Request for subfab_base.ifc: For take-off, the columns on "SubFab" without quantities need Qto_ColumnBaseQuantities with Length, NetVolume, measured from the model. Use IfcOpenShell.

First a look at what the model holds.

```python
import ifcopenshell
import ifcopenshell.util.element
import ifcopenshell.util.unit

model = ifcopenshell.open("subfab_base.ifc")
print(model.schema)
for unit_type in ("LENGTHUNIT", "AREAUNIT", "VOLUMEUNIT"):
    print(unit_type, ifcopenshell.util.unit.calculate_unit_scale(model, unit_type))
storey = next(s for s in model.by_type("IfcBuildingStorey") if s.Name == "SubFab")
columns = [e for e in ifcopenshell.util.element.get_decomposition(storey) if e.is_a("IfcColumn")]
for e in sorted(columns, key=lambda e: e.id()):
    print(e.id(), e.is_a(), e.Name, list(ifcopenshell.util.element.get_psets(e, qtos_only=True)), sep=" | ")
```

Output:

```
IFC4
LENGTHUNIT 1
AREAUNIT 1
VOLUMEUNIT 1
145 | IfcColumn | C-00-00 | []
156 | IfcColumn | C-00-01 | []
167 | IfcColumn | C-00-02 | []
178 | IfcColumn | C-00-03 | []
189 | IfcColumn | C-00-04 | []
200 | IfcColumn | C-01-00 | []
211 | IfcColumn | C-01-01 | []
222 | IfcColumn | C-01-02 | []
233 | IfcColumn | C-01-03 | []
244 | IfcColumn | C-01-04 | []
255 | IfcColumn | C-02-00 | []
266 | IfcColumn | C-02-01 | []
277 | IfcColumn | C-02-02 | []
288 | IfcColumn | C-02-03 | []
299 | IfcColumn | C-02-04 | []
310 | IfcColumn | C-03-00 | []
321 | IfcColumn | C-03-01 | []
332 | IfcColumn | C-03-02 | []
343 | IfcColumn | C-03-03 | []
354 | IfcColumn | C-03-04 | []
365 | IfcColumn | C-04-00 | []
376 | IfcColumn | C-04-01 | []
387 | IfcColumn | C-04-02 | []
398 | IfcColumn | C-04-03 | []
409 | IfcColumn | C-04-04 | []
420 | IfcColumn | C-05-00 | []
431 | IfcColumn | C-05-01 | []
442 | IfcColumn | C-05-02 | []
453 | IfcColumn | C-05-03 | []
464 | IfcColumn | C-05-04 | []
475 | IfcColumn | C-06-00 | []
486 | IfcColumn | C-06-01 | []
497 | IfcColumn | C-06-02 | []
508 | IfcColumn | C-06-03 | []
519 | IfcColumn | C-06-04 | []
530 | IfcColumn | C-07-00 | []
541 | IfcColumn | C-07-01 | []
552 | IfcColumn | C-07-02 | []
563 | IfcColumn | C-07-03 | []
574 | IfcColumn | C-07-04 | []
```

```python
import ifcopenshell
import ifcopenshell.api.pset
import ifcopenshell.geom
import ifcopenshell.util.element
import ifcopenshell.util.shape
import ifcopenshell.util.unit

model = ifcopenshell.open("subfab_base.ifc")
unit_scale = ifcopenshell.util.unit.calculate_unit_scale(model)
volume_scale = ifcopenshell.util.unit.calculate_unit_scale(model, "VOLUMEUNIT")
settings = ifcopenshell.geom.settings()

storey = next(s for s in model.by_type("IfcBuildingStorey") if s.Name == "SubFab")
columns = [e for e in ifcopenshell.util.element.get_decomposition(storey) if e.is_a("IfcColumn")]

for e in sorted(columns, key=lambda e: e.id()):
    if ifcopenshell.util.element.get_psets(e, qtos_only=True, should_inherit=False):
        continue
    # Geometry comes back in metres, in the element's own axes.
    shape = ifcopenshell.geom.create_shape(settings, e)
    values = {
        "Length": ifcopenshell.util.shape.get_z(shape.geometry) / unit_scale,
        "NetVolume": ifcopenshell.util.shape.get_volume(shape.geometry) / volume_scale,
    }
    qto = ifcopenshell.api.pset.add_qto(model, product=e, name="Qto_ColumnBaseQuantities")
    ifcopenshell.api.pset.edit_qto(model, qto=qto, properties=values)
    print(e.id(), {k: round(v, 3) for k, v in values.items()})

model.write("subfab_base_v2.ifc")
```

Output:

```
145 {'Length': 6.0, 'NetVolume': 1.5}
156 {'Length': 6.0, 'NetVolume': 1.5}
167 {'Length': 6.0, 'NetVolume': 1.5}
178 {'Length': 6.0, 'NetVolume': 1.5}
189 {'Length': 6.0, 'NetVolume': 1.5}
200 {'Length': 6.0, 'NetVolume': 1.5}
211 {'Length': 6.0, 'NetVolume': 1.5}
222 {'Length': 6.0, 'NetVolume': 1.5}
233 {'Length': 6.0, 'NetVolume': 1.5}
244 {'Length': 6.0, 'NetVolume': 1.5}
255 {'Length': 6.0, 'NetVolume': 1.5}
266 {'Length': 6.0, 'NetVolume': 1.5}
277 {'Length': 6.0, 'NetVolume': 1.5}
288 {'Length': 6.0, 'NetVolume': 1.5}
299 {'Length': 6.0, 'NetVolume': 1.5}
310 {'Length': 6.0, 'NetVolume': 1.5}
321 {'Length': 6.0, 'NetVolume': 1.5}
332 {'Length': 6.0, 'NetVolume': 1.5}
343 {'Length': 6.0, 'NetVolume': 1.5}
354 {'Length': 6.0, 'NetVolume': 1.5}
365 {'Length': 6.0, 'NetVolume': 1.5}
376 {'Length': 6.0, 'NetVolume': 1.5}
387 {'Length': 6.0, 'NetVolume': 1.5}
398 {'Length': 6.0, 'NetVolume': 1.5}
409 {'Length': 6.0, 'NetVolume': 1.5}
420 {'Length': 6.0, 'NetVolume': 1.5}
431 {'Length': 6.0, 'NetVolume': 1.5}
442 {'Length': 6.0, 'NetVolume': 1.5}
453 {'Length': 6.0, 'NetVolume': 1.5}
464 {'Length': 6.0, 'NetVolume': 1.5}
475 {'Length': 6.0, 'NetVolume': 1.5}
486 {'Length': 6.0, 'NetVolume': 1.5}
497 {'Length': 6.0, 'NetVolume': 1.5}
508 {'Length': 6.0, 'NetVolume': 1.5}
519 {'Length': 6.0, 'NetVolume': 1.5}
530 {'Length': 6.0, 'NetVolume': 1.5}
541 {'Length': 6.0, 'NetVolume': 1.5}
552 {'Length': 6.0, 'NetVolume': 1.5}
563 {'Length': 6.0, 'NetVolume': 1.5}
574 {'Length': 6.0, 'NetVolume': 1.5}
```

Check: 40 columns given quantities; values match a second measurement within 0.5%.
